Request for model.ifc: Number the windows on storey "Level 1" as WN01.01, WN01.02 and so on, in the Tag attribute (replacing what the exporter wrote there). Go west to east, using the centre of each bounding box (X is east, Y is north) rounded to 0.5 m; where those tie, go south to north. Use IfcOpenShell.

First a look at what the model holds.

```python
import ifcopenshell
import ifcopenshell.util.element
import ifcopenshell.util.placement

model = ifcopenshell.open("model.ifc")
print(model.schema)
storey = next(s for s in model.by_type("IfcBuildingStorey") if s.Name == "Level 1")
windows = [e for e in ifcopenshell.util.element.get_decomposition(storey) if e.is_a("IfcWindow")]
for e in sorted(windows, key=lambda e: e.id()):
    origin = ifcopenshell.util.placement.get_local_placement(e.ObjectPlacement)[:3, 3]
    print(e.id(), e.Tag, e.Name, origin.round(2) + 0.0, sep=" | ")
```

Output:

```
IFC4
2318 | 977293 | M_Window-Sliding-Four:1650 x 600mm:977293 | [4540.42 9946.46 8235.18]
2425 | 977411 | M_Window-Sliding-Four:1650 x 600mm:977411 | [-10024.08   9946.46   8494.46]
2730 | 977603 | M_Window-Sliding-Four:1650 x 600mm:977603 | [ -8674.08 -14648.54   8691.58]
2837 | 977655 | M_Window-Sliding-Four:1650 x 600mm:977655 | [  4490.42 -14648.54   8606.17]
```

```python
import ifcopenshell
import ifcopenshell.geom
import ifcopenshell.util.element
import ifcopenshell.util.shape

model = ifcopenshell.open("model.ifc")
settings = ifcopenshell.geom.settings()
settings.set("use-world-coords", True)


def centre(element):
    shape = ifcopenshell.geom.create_shape(settings, element)
    return ifcopenshell.util.shape.get_bbox_centroid(shape.geometry)


storey = next(s for s in model.by_type("IfcBuildingStorey") if s.Name == "Level 1")
windows = [e for e in ifcopenshell.util.element.get_decomposition(storey) if e.is_a("IfcWindow")]

# Insertion points can sit at a corner or the storey origin, so sort by the geometry (in metres).
centres = {e: centre(e) for e in windows}
windows.sort(key=lambda e: (round(centres[e][0] / 0.5), centres[e][1]))

for i, e in enumerate(windows, start=1):
    number = f"WN01.{i:02d}"
    e.Tag = number
    print(e.id(), number)

model.write("model_edited.ifc")
```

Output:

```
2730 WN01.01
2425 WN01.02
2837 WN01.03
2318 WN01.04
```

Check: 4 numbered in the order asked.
